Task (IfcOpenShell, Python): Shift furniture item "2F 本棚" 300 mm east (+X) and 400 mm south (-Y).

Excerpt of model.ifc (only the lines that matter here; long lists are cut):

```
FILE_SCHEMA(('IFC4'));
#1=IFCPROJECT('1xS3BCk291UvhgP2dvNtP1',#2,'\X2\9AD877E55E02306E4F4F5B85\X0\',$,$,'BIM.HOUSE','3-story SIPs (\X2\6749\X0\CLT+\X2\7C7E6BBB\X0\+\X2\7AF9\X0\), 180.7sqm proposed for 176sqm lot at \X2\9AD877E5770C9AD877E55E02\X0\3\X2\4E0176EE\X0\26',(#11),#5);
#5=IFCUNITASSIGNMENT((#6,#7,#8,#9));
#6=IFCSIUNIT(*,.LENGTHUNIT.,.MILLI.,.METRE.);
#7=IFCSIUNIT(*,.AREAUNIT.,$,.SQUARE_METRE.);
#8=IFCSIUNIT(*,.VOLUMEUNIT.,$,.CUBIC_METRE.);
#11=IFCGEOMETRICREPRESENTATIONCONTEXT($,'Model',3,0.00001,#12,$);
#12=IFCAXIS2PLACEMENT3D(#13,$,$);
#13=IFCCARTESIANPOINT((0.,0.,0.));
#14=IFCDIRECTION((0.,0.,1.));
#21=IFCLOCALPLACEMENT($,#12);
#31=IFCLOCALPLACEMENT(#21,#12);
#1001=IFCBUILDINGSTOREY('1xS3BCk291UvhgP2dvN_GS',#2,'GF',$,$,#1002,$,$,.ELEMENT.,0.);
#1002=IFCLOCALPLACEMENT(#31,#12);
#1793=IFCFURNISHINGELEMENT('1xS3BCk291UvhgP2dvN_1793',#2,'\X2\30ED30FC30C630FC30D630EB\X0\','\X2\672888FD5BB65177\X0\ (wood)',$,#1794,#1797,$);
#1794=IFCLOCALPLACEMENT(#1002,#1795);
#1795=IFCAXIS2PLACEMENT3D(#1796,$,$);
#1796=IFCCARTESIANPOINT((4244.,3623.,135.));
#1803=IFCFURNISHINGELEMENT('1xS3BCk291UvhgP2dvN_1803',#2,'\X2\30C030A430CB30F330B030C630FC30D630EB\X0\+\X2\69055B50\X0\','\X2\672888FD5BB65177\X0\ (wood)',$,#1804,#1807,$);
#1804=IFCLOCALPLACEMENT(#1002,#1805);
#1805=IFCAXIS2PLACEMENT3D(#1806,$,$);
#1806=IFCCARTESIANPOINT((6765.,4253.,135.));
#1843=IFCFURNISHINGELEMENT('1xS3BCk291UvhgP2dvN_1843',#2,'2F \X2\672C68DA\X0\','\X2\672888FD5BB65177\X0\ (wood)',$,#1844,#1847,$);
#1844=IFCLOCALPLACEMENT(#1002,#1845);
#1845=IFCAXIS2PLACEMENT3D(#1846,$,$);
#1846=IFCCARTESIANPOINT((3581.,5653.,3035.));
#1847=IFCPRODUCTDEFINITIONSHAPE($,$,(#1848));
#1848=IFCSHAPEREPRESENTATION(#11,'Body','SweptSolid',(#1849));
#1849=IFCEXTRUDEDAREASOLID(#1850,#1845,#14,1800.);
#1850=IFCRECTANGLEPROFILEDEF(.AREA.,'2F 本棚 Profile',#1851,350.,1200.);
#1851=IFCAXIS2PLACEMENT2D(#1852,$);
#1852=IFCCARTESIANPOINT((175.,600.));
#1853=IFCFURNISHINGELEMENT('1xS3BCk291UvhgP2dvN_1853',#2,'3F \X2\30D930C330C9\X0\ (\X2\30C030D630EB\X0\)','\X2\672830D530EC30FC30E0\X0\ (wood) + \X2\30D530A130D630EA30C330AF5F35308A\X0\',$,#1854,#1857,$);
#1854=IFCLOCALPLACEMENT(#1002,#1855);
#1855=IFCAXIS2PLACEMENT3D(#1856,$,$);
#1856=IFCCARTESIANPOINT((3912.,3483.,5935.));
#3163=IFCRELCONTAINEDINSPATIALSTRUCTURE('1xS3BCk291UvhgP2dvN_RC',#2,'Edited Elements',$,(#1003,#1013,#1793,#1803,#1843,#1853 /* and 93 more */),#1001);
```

```python
import ifcopenshell
import ifcopenshell.api.geometry
import ifcopenshell.util.placement
import ifcopenshell.util.unit

model = ifcopenshell.open("model.ifc")
unit_scale = ifcopenshell.util.unit.calculate_unit_scale(model)

item = model.by_guid("1xS3BCk291UvhgP2dvN_1843")
matrix = ifcopenshell.util.placement.get_local_placement(item.ObjectPlacement)
matrix[0, 3] += 0.3 / unit_scale
matrix[1, 3] -= 0.4 / unit_scale
ifcopenshell.api.geometry.edit_object_placement(model, product=item, matrix=matrix, is_si=False)

print(ifcopenshell.util.placement.get_local_placement(item.ObjectPlacement).round(3) + 0.0)

model.write("model_v2.ifc")
```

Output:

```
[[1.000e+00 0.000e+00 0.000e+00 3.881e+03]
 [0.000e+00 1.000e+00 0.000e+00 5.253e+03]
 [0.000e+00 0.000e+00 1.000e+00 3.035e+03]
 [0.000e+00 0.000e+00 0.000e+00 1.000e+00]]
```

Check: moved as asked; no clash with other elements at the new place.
